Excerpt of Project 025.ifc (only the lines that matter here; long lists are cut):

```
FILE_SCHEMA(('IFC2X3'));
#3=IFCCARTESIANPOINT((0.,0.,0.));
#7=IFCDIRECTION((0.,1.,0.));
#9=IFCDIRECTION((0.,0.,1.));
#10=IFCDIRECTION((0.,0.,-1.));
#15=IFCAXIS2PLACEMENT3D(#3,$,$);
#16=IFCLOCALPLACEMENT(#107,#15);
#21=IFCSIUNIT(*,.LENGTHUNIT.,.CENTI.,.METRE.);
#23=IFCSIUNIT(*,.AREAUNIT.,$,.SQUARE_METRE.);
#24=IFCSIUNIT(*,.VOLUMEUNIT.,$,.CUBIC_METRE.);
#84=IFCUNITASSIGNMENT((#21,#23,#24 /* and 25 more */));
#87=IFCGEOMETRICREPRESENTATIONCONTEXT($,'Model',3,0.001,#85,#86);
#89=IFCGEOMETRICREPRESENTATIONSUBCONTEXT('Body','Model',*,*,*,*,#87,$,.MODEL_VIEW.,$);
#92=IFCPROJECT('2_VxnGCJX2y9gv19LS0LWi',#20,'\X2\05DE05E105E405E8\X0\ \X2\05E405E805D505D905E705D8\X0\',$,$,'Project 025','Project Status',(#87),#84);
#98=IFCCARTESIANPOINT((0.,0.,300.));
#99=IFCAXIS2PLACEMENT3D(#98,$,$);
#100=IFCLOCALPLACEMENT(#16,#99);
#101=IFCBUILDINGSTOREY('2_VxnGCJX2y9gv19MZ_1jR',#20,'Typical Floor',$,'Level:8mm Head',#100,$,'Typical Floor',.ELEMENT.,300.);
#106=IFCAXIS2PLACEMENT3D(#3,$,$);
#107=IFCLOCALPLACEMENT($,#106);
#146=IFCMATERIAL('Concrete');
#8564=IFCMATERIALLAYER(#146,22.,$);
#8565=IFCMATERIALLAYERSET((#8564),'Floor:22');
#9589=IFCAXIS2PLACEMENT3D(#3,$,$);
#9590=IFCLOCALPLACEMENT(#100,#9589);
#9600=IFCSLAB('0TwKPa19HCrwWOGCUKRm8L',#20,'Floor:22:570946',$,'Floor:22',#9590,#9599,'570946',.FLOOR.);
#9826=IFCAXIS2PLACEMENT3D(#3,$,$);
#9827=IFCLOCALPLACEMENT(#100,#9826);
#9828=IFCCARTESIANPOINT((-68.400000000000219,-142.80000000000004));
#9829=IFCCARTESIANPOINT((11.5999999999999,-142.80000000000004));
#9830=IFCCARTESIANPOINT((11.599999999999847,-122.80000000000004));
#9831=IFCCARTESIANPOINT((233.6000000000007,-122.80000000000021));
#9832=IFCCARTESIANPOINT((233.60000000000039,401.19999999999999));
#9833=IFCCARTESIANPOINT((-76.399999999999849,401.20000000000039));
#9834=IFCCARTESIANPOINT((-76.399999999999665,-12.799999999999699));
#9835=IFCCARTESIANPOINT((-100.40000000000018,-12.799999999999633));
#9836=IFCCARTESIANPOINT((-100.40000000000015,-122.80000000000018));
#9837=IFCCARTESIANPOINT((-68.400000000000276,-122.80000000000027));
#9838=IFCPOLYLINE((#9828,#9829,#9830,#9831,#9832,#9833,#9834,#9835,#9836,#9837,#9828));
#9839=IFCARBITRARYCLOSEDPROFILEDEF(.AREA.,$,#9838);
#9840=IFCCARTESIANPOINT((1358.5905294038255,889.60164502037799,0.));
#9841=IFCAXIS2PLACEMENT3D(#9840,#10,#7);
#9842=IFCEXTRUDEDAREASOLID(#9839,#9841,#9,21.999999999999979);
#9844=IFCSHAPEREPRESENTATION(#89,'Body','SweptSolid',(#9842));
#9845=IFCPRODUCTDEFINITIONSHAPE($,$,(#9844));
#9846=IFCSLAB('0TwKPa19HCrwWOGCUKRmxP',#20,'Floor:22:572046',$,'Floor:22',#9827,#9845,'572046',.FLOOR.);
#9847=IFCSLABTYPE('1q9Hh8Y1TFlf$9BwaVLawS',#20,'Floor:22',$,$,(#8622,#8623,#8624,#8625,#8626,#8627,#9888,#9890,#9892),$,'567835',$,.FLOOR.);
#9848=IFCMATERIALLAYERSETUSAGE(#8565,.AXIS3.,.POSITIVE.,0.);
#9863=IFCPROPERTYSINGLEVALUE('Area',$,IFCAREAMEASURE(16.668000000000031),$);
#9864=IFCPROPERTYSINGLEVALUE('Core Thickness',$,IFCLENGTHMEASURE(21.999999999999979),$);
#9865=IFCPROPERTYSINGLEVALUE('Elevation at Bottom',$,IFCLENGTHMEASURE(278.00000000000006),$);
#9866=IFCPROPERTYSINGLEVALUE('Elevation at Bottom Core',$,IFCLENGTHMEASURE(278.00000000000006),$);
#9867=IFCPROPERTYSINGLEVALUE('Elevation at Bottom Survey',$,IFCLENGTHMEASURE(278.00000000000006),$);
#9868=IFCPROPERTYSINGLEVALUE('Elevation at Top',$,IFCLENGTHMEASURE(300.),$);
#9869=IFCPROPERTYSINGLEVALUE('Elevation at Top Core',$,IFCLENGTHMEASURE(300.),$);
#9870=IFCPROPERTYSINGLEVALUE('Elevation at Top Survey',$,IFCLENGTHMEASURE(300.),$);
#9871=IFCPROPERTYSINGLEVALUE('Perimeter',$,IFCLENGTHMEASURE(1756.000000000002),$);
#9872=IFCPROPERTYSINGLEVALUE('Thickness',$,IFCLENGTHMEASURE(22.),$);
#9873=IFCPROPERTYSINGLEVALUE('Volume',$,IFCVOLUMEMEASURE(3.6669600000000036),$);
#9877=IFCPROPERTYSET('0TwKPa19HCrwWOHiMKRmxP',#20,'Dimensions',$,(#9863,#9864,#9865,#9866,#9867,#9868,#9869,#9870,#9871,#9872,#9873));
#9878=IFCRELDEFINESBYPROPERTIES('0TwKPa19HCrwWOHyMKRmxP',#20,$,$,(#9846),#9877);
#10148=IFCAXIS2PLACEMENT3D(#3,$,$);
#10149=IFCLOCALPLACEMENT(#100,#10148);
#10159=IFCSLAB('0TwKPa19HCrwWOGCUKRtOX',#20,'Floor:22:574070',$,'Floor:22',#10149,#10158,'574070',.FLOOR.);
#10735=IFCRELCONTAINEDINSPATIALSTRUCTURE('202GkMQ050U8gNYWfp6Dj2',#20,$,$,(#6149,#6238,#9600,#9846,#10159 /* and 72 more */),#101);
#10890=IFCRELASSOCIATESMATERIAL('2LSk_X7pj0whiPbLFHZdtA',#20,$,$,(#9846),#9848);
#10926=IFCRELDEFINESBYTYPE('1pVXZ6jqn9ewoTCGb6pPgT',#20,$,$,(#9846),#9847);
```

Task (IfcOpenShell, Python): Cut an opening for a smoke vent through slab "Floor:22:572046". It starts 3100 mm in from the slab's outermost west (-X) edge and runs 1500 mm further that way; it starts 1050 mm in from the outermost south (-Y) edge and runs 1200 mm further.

```python
import numpy as np
import ifcopenshell
import ifcopenshell.api.feature
import ifcopenshell.api.geometry
import ifcopenshell.api.pset
import ifcopenshell.api.root
import ifcopenshell.geom
import ifcopenshell.util.element
import ifcopenshell.util.placement
import ifcopenshell.util.representation
import ifcopenshell.util.shape
import ifcopenshell.util.unit

model = ifcopenshell.open("Project 025.ifc")
unit_scale = ifcopenshell.util.unit.calculate_unit_scale(model)
area_scale = ifcopenshell.util.unit.calculate_unit_scale(model, "AREAUNIT")
volume_scale = ifcopenshell.util.unit.calculate_unit_scale(model, "VOLUMEUNIT")
settings = ifcopenshell.geom.settings()


def volume(element):
    """Net volume in cubic metres, openings subtracted."""
    shape = ifcopenshell.geom.create_shape(settings, element)
    return ifcopenshell.util.shape.get_volume(shape.geometry)


slab = model.by_guid("0TwKPa19HCrwWOGCUKRmxP")
before = volume(slab)

# Extent in the slab's own axes, in metres. The edges named are its -X and -Y sides.
slab_shape = ifcopenshell.geom.create_shape(settings, slab)
vertices = ifcopenshell.util.shape.get_vertices(slab_shape.geometry)
x_min, y_min, bottom = vertices.min(axis=0)
top = vertices[:, 2].max()

opening = ifcopenshell.api.root.create_entity(model, ifc_class="IfcOpeningElement", name="Smoke vent opening")
context = ifcopenshell.util.representation.get_context(model, "Model", "Body", "MODEL_VIEW")
width, depth = 1.5, 1.2
outline = [(0.0, 0.0), (width, 0.0), (width, depth), (0.0, depth), (0.0, 0.0)]
# Overshoot both faces by 50 mm so the cut is clean.
shape = ifcopenshell.api.geometry.add_slab_representation(
    model, context=context, depth=top - bottom + 0.1, polyline=outline
)
ifcopenshell.api.geometry.assign_representation(model, product=opening, representation=shape)

matrix = ifcopenshell.util.placement.get_local_placement(slab.ObjectPlacement)
matrix[:, 3] = matrix @ np.append(np.array([x_min + 3.1, y_min + 1.05, bottom - 0.05]) / unit_scale, 1.0)
ifcopenshell.api.geometry.edit_object_placement(model, product=opening, matrix=matrix, is_si=False)
ifcopenshell.api.feature.add_feature(model, feature=opening, element=slab)

after = volume(slab)

# Update the slab's stored quantities.
pset = model.by_id(ifcopenshell.util.element.get_pset(slab, "Dimensions", should_inherit=False)["id"])
ifcopenshell.api.pset.edit_pset(model, pset=pset, properties={
    "Area": model.create_entity("IfcAreaMeasure", after / (top - bottom) / area_scale),
    "Volume": model.create_entity("IfcVolumeMeasure", after / volume_scale),
})

print(f"slab volume {before:.3f} -> {after:.3f} m3")

model.write("Project 025_v2.ifc")
```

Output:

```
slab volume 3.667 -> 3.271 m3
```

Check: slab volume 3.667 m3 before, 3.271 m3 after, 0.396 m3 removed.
